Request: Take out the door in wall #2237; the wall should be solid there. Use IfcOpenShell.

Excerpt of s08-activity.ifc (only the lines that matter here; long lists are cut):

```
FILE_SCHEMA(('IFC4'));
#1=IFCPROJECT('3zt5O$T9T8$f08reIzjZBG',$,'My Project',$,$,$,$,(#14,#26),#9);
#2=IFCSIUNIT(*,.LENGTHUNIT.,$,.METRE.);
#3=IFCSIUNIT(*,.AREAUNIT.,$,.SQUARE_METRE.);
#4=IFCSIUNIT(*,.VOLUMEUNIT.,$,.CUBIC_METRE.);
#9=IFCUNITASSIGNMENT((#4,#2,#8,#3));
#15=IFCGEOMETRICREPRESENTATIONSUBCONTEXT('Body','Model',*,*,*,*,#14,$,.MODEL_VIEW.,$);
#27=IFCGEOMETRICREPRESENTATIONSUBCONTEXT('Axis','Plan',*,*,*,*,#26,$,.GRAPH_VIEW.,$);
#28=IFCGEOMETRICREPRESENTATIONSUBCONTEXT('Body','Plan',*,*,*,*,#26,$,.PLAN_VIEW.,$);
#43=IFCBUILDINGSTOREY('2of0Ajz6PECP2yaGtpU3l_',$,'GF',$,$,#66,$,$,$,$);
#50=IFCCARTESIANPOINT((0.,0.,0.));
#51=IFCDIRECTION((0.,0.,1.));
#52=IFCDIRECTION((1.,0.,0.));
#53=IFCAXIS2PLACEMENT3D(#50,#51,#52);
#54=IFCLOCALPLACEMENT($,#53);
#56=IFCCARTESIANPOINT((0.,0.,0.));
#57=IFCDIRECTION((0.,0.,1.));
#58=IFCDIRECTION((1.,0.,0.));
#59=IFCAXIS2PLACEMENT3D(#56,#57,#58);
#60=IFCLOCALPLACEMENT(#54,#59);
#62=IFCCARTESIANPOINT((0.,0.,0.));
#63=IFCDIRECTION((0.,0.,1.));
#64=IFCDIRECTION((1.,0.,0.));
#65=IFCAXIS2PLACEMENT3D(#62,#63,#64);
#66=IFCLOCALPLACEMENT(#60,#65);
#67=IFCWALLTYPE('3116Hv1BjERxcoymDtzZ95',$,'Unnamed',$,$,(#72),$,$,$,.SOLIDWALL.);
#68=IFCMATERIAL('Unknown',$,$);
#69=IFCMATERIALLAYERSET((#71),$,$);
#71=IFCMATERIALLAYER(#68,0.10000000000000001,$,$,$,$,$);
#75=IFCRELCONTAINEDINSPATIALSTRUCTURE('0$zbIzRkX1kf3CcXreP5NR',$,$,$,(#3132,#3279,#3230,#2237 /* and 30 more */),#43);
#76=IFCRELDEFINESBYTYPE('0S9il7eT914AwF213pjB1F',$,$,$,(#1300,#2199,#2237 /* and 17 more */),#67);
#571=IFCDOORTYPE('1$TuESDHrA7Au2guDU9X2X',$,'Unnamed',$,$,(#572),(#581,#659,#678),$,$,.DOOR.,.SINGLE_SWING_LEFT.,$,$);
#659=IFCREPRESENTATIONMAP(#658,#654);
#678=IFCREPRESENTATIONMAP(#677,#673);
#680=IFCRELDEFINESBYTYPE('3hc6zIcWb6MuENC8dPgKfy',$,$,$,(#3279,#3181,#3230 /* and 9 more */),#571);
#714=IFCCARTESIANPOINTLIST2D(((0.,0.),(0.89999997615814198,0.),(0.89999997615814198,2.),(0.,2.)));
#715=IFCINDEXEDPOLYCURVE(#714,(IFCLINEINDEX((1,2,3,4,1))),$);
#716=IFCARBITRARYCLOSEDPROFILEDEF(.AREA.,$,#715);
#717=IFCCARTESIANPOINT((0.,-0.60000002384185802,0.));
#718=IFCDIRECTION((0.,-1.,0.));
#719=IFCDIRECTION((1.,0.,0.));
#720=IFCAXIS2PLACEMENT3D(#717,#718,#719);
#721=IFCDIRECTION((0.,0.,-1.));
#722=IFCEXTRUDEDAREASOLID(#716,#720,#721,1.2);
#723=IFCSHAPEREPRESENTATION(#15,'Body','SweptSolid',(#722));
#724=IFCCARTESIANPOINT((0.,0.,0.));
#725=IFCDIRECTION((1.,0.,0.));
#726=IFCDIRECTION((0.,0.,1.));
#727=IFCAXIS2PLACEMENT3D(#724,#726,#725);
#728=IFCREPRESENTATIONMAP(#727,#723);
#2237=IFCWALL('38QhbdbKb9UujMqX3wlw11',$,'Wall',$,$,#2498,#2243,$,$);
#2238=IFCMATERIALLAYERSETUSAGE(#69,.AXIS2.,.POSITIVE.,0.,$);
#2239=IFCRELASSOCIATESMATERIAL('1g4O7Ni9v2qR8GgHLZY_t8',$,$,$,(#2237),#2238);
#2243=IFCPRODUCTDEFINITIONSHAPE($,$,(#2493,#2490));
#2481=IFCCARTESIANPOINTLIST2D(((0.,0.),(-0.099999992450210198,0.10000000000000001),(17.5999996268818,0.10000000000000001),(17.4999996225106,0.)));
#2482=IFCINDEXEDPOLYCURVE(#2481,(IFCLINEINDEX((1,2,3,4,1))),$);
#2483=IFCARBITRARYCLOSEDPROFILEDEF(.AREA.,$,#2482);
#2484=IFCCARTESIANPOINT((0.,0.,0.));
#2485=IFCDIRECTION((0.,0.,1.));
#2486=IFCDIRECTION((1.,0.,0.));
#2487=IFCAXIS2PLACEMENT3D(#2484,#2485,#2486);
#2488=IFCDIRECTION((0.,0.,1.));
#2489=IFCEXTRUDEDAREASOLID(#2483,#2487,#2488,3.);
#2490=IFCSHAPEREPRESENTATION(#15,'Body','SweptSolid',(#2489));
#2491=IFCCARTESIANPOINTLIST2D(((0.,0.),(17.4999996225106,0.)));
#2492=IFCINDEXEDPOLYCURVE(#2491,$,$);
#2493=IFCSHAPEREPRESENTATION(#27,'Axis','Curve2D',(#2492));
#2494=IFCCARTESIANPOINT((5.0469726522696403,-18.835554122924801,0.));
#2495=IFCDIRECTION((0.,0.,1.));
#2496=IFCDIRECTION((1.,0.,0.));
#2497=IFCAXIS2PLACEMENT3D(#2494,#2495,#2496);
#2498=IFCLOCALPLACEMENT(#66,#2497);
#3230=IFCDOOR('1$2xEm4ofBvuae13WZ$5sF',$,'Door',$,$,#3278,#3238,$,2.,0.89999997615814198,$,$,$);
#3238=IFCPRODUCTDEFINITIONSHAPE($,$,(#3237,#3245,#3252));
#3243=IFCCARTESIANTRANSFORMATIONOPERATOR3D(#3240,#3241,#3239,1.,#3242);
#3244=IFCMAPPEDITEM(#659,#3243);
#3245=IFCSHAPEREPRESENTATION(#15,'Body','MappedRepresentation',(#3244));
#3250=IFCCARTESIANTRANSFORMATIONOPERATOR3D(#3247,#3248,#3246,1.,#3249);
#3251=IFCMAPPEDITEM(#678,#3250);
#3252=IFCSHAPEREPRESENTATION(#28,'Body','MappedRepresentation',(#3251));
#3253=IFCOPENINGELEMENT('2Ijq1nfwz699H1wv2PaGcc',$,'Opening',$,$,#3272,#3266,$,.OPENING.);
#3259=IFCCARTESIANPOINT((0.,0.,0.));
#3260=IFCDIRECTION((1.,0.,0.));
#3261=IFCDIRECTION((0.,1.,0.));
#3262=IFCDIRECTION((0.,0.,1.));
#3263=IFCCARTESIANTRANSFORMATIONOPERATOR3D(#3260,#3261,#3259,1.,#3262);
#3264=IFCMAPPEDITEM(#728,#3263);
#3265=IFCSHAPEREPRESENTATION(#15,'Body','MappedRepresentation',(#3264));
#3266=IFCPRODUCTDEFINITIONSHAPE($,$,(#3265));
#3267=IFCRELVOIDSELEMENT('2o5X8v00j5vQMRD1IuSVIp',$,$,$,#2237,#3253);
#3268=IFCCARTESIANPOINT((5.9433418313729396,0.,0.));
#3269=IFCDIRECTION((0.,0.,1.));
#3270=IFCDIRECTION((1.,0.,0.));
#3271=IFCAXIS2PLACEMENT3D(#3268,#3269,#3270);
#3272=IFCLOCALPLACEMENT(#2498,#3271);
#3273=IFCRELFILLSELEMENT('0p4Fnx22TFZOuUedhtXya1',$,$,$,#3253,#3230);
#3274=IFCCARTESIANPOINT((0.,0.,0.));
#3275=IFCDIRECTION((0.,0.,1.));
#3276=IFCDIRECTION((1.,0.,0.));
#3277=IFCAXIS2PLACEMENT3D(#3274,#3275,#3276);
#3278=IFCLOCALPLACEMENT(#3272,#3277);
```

```python
import ifcopenshell
import ifcopenshell.api.feature
import ifcopenshell.api.root
import ifcopenshell.geom
import ifcopenshell.util.shape

model = ifcopenshell.open("s08-activity.ifc")
settings = ifcopenshell.geom.settings()


def volume(element):
    """Net volume in cubic metres, openings subtracted."""
    shape = ifcopenshell.geom.create_shape(settings, element)
    return ifcopenshell.util.shape.get_volume(shape.geometry)


door = model.by_id(3230)
opening = door.FillsVoids[0].RelatingOpeningElement
wall = opening.VoidsElements[0].RelatingBuildingElement
before = volume(wall)

ifcopenshell.api.root.remove_product(model, product=door)
ifcopenshell.api.feature.remove_feature(model, feature=opening)

after = volume(wall)

print(f"wall volume {before:.3f} -> {after:.3f} m3")

model.write("s08-activity_updated.ifc")
```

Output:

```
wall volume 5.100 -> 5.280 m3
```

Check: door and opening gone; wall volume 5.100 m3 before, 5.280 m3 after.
